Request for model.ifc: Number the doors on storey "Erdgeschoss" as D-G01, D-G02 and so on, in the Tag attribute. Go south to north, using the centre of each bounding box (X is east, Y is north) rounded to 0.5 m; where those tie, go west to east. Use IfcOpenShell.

First a look at what the model holds.

```python
import ifcopenshell
import ifcopenshell.util.element
import ifcopenshell.util.placement

model = ifcopenshell.open("model.ifc")
print(model.schema)
storey = next(s for s in model.by_type("IfcBuildingStorey") if s.Name == "Erdgeschoss")
doors = [e for e in ifcopenshell.util.element.get_decomposition(storey) if e.is_a("IfcDoor")]
for e in sorted(doors, key=lambda e: e.id()):
    origin = ifcopenshell.util.placement.get_local_placement(e.ObjectPlacement)[:3, 3]
    print(e.id(), e.Tag, e.Name, origin.round(2) + 0.0, sep=" | ")
```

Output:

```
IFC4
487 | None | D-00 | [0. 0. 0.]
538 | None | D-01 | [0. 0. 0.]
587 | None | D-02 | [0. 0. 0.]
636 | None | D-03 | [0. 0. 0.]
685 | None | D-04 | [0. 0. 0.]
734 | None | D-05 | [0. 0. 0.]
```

```python
import ifcopenshell
import ifcopenshell.geom
import ifcopenshell.util.element
import ifcopenshell.util.shape

model = ifcopenshell.open("model.ifc")
settings = ifcopenshell.geom.settings()
settings.set("use-world-coords", True)


def centre(element):
    shape = ifcopenshell.geom.create_shape(settings, element)
    return ifcopenshell.util.shape.get_bbox_centroid(shape.geometry)


storey = next(s for s in model.by_type("IfcBuildingStorey") if s.Name == "Erdgeschoss")
doors = [e for e in ifcopenshell.util.element.get_decomposition(storey) if e.is_a("IfcDoor")]

# Insertion points can sit at a corner or the storey origin, so sort by the geometry (in metres).
centres = {e: centre(e) for e in doors}
doors.sort(key=lambda e: (round(centres[e][1] / 0.5), centres[e][0]))

for i, e in enumerate(doors, start=1):
    number = f"D-G{i:02d}"
    e.Tag = number
    print(e.id(), number)

model.write("model_updated.ifc")
```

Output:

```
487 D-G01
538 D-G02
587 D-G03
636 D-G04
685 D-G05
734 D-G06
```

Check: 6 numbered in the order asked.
